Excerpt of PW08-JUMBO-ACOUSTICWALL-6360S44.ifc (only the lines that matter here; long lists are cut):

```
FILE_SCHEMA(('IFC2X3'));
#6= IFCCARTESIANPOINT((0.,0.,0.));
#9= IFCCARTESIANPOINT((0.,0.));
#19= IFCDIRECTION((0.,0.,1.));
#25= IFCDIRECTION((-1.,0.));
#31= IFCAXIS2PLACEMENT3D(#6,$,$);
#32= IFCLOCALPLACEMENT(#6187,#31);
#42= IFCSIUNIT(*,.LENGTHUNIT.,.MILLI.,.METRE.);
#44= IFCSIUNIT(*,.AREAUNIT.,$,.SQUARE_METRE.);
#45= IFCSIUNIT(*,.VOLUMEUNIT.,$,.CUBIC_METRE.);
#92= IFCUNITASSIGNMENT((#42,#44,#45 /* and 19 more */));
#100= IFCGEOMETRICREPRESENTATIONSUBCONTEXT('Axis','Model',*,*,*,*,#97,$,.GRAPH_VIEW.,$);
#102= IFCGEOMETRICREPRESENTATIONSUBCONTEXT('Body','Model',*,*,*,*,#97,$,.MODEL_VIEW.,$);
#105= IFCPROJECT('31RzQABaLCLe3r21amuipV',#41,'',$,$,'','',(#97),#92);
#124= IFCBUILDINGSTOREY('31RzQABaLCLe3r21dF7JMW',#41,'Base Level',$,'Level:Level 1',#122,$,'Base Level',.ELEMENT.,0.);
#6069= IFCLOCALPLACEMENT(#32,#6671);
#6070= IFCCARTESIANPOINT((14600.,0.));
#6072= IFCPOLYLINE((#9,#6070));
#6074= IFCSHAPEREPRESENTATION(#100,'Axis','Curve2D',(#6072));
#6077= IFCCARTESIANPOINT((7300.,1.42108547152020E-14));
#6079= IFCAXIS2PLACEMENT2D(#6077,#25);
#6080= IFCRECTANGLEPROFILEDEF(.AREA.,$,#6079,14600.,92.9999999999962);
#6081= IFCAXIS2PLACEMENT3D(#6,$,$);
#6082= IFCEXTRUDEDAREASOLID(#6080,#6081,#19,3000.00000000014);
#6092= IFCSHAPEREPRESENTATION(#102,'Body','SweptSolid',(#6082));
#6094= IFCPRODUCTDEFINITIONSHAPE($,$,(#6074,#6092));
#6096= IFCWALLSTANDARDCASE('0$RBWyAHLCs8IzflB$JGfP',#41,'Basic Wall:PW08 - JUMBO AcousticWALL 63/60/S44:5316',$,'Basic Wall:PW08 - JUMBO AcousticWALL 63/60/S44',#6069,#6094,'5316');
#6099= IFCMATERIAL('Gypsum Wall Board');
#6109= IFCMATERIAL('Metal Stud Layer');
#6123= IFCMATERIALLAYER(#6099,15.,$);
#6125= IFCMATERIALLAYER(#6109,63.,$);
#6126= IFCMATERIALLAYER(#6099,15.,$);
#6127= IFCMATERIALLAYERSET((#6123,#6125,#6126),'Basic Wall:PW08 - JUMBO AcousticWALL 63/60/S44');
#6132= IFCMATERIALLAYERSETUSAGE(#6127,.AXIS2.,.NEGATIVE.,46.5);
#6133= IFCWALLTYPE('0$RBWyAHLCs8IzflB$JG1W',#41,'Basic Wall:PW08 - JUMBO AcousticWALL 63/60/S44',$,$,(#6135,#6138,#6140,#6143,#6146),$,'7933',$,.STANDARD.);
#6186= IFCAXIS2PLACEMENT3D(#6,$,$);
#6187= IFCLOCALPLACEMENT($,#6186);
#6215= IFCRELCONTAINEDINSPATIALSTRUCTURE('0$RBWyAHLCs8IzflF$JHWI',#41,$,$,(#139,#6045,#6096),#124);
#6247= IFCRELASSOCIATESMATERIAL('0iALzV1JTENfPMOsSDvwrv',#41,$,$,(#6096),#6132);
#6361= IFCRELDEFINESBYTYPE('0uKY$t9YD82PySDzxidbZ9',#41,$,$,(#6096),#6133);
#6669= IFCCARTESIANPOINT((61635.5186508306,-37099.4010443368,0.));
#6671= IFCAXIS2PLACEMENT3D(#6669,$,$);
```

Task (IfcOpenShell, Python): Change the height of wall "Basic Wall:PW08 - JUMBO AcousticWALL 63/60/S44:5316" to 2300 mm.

```python
import ifcopenshell
import ifcopenshell.geom
import ifcopenshell.util.representation
import ifcopenshell.util.shape
import ifcopenshell.util.unit

model = ifcopenshell.open("PW08-JUMBO-ACOUSTICWALL-6360S44.ifc")
unit_scale = ifcopenshell.util.unit.calculate_unit_scale(model)
settings = ifcopenshell.geom.settings()


def volume(element):
    """Net volume in cubic metres, openings subtracted."""
    shape = ifcopenshell.geom.create_shape(settings, element)
    return ifcopenshell.util.shape.get_volume(shape.geometry)


wall = model.by_guid("0$RBWyAHLCs8IzflB$JGfP")
before = volume(wall)

body = ifcopenshell.util.representation.get_representation(wall, "Model", "Body")
solid = body.Items[0]
old_height = solid.Depth
solid.Depth = 2.3 / unit_scale
after = volume(wall)

print(f"height {old_height:g} -> {solid.Depth:g}, volume {before:.3f} -> {after:.3f} m3")

model.write("PW08-JUMBO-ACOUSTICWALL-6360S44_updated.ifc")
```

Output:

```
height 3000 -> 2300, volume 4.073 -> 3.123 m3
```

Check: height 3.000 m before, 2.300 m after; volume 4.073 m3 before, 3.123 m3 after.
